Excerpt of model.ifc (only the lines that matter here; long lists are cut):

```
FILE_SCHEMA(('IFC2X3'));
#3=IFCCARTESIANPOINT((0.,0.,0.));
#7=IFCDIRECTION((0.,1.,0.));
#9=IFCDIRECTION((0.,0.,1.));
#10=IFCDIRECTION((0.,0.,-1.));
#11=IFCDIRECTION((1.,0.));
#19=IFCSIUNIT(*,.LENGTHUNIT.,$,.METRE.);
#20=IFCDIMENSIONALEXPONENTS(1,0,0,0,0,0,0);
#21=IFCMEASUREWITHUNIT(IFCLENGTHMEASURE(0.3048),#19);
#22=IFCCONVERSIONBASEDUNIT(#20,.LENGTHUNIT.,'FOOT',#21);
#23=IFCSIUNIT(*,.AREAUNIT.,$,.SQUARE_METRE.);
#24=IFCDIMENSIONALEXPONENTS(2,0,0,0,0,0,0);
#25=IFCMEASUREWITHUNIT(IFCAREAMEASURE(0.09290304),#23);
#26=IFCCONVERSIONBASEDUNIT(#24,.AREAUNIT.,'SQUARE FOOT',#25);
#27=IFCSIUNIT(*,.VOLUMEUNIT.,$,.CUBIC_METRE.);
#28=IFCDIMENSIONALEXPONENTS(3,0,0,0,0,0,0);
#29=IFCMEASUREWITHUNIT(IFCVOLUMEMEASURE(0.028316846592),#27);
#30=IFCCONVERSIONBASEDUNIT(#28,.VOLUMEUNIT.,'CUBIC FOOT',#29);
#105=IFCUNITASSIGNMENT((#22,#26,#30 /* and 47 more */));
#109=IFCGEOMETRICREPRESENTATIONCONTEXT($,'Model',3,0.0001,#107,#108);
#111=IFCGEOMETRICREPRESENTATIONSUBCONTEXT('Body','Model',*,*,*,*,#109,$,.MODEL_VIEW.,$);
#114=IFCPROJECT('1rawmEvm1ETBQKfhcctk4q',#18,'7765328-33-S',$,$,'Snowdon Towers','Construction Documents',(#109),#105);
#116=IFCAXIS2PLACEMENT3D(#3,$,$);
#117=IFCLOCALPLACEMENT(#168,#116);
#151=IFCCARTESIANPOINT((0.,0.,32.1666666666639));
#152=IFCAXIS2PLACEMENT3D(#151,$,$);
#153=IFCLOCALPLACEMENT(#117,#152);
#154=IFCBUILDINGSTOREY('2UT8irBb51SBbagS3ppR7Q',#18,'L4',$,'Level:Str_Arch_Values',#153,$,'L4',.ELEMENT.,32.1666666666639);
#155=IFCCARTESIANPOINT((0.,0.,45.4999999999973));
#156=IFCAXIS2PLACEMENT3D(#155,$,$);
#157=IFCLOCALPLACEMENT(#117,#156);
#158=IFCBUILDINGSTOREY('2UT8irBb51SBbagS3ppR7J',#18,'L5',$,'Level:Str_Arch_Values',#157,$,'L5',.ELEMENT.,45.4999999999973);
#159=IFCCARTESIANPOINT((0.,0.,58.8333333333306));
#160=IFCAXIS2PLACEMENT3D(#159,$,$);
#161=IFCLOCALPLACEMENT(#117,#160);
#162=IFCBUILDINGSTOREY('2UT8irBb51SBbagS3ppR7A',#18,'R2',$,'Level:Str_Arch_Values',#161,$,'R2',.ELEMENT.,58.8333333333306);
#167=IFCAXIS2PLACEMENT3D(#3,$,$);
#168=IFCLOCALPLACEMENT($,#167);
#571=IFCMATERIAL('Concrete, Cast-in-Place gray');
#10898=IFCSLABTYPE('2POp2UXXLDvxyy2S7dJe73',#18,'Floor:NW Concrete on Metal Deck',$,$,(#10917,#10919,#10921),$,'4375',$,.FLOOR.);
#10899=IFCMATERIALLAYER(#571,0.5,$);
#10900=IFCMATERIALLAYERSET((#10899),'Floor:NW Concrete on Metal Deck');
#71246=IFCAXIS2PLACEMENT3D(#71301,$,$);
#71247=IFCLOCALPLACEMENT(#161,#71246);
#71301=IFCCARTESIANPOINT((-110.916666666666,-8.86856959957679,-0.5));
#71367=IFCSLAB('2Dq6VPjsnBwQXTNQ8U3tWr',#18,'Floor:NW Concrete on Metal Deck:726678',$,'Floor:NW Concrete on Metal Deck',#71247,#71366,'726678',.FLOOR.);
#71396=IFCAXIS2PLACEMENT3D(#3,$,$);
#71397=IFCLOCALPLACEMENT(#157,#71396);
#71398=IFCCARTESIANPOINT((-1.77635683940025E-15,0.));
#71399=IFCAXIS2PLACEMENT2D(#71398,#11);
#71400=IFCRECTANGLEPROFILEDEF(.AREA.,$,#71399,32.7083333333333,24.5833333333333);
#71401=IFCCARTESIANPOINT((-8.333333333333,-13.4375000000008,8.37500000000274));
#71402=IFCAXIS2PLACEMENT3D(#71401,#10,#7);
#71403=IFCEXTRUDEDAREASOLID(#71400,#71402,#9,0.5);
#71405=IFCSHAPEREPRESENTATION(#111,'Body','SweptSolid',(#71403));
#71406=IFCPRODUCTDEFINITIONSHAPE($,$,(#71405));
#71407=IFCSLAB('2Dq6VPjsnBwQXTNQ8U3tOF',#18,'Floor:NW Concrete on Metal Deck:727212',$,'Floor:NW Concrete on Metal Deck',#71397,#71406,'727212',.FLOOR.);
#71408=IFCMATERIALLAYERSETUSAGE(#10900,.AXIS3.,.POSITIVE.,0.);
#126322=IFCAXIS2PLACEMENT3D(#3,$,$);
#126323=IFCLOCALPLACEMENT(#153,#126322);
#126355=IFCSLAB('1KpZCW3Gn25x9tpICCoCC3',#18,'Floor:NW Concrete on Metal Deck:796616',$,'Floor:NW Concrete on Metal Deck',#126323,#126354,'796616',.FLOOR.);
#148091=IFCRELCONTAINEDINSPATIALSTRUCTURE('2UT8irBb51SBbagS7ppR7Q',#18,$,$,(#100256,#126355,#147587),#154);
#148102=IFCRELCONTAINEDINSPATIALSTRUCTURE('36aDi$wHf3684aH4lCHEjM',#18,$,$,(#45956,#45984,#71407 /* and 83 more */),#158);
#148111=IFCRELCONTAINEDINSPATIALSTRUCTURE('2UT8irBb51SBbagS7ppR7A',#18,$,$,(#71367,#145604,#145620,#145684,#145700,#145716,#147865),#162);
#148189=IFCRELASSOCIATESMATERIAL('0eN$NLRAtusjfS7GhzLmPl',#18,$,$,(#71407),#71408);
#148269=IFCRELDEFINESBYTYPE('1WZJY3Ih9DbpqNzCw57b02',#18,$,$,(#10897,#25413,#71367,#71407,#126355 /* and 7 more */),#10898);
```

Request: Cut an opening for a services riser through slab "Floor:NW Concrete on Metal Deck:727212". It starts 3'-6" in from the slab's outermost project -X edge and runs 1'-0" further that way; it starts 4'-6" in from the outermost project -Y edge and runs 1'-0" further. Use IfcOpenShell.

```python
import numpy as np
import ifcopenshell
import ifcopenshell.api.feature
import ifcopenshell.api.geometry
import ifcopenshell.api.root
import ifcopenshell.geom
import ifcopenshell.util.placement
import ifcopenshell.util.representation
import ifcopenshell.util.shape
import ifcopenshell.util.unit

model = ifcopenshell.open("model.ifc")
unit_scale = ifcopenshell.util.unit.calculate_unit_scale(model)
settings = ifcopenshell.geom.settings()


def volume(element):
    """Net volume in cubic metres, openings subtracted."""
    shape = ifcopenshell.geom.create_shape(settings, element)
    return ifcopenshell.util.shape.get_volume(shape.geometry)


slab = model.by_guid("2Dq6VPjsnBwQXTNQ8U3tOF")
before = volume(slab)

# Extent in the slab's own axes, in metres. The edges named are its -X and -Y sides.
slab_shape = ifcopenshell.geom.create_shape(settings, slab)
vertices = ifcopenshell.util.shape.get_vertices(slab_shape.geometry)
x_min, y_min, bottom = vertices.min(axis=0)
top = vertices[:, 2].max()

opening = ifcopenshell.api.root.create_entity(model, ifc_class="IfcOpeningElement", name="Services riser opening")
context = ifcopenshell.util.representation.get_context(model, "Model", "Body", "MODEL_VIEW")
width, depth = 0.3048, 0.3048
outline = [(0.0, 0.0), (width, 0.0), (width, depth), (0.0, depth), (0.0, 0.0)]
# Overshoot both faces by 50 mm so the cut is clean.
shape = ifcopenshell.api.geometry.add_slab_representation(
    model, context=context, depth=top - bottom + 0.1, polyline=outline
)
ifcopenshell.api.geometry.assign_representation(model, product=opening, representation=shape)

matrix = ifcopenshell.util.placement.get_local_placement(slab.ObjectPlacement)
matrix[:, 3] = matrix @ np.append(np.array([x_min + 1.0668, y_min + 1.3716, bottom - 0.05]) / unit_scale, 1.0)
ifcopenshell.api.geometry.edit_object_placement(model, product=opening, matrix=matrix, is_si=False)
ifcopenshell.api.feature.add_feature(model, feature=opening, element=slab)

after = volume(slab)

print(f"slab volume {before:.3f} -> {after:.3f} m3")

model.write("model-out.ifc")
```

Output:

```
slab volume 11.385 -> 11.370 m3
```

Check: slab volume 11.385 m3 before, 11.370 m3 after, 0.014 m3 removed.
